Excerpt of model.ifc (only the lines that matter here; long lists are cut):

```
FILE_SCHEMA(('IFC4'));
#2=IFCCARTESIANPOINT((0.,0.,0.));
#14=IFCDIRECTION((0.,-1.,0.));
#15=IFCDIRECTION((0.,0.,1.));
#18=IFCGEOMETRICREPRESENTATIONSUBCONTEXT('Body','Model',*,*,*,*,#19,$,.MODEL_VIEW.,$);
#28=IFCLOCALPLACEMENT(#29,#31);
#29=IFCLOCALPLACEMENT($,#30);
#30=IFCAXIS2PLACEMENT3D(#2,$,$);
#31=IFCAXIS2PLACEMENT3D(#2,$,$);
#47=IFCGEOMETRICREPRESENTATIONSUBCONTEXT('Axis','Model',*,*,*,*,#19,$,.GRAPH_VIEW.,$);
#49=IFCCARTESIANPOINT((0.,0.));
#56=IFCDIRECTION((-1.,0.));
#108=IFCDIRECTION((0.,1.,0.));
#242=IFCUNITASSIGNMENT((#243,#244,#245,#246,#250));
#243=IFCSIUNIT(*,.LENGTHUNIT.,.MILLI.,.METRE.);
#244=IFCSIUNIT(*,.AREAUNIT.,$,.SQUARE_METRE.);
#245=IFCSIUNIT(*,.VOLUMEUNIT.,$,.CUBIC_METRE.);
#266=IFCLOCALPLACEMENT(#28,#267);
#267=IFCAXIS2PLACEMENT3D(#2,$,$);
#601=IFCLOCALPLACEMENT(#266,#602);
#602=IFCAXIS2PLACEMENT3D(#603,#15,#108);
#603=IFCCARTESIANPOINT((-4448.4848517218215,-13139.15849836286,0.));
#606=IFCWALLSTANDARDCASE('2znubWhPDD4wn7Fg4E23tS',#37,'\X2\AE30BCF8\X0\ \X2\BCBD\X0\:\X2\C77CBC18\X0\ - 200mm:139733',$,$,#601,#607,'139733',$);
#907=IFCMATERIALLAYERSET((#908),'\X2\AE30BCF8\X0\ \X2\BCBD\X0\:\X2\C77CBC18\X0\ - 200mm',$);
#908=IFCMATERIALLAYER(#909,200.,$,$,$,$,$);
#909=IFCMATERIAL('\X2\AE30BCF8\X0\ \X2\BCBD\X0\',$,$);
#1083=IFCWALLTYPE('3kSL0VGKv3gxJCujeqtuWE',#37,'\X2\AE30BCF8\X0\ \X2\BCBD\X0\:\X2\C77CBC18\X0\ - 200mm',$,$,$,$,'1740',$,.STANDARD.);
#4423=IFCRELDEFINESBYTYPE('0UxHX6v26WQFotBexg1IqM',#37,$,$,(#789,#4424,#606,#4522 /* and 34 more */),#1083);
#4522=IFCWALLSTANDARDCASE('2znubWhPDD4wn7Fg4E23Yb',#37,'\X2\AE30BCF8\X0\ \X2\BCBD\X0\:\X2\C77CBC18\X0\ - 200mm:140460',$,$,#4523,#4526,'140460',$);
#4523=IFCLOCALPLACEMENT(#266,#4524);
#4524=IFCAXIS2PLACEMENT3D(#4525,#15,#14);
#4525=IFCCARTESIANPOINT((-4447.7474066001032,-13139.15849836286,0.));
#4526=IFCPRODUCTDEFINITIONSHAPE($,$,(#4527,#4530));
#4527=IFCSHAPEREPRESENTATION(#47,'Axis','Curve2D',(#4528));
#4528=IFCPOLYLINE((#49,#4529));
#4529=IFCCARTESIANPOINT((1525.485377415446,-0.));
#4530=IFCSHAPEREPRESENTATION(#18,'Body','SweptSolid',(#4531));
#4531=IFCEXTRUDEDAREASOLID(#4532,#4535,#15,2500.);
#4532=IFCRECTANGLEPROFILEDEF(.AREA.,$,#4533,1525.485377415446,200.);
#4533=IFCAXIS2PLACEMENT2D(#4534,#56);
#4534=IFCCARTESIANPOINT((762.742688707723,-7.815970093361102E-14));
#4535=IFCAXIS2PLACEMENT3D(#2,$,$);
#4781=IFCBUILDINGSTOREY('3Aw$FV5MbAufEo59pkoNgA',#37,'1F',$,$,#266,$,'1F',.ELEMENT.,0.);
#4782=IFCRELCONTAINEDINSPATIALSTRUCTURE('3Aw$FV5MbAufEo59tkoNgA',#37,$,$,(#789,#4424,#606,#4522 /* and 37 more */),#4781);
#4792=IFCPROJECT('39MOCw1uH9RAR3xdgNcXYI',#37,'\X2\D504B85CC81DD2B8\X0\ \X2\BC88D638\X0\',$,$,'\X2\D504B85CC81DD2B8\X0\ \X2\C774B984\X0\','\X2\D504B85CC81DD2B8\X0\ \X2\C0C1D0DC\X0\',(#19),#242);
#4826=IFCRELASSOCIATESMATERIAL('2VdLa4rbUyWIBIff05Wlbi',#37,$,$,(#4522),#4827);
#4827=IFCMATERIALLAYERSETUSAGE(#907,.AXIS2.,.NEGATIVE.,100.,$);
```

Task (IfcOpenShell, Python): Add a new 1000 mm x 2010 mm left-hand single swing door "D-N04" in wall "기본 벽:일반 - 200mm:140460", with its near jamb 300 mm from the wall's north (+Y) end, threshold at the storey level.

```python
import numpy as np
import ifcopenshell
import ifcopenshell.api.feature
import ifcopenshell.api.geometry
import ifcopenshell.api.root
import ifcopenshell.api.spatial
import ifcopenshell.geom
import ifcopenshell.util.element
import ifcopenshell.util.placement
import ifcopenshell.util.representation
import ifcopenshell.util.shape
import ifcopenshell.util.unit

model = ifcopenshell.open("model.ifc")
unit_scale = ifcopenshell.util.unit.calculate_unit_scale(model)
settings = ifcopenshell.geom.settings()


def volume(element):
    """Net volume in cubic metres, openings subtracted."""
    shape = ifcopenshell.geom.create_shape(settings, element)
    return ifcopenshell.util.shape.get_volume(shape.geometry)


wall = model.by_id(4522)
storey = ifcopenshell.util.element.get_container(wall, ifc_class="IfcBuildingStorey")
context = ifcopenshell.util.representation.get_context(model, "Model", "Body", "MODEL_VIEW")
before = volume(wall)

width, height, from_end, sill = 1, 2.01, 0.3, 0.0  # metres

# The wall runs along its own X axis, and the end named is its -X end.
wall_shape = ifcopenshell.geom.create_shape(settings, wall)
x, y, z = ifcopenshell.util.shape.get_vertices(wall_shape.geometry).T
start = x.min() + from_end
face, thickness = float(y.min()), float(y.max() - y.min())
wall_matrix = ifcopenshell.util.placement.get_local_placement(wall.ObjectPlacement)
level = ifcopenshell.util.placement.get_local_placement(storey.ObjectPlacement)[2, 3]


def in_wall(x, y):
    """Placement at x, y metres in the wall's axes, at sill height."""
    matrix = wall_matrix.copy()
    matrix[:, 3] = wall_matrix @ np.array([x / unit_scale, y / unit_scale, 0.0, 1.0])
    matrix[2, 3] = level + sill / unit_scale
    return matrix


# Opening: a box that overshoots both wall faces by 50 mm.
opening = ifcopenshell.api.root.create_entity(model, ifc_class="IfcOpeningElement", predefined_type="OPENING")
box = ifcopenshell.api.geometry.add_wall_representation(
    model, context=context, length=width, height=height, thickness=thickness + 0.1
)
ifcopenshell.api.geometry.assign_representation(model, product=opening, representation=box)
ifcopenshell.api.geometry.edit_object_placement(model, product=opening, matrix=in_wall(start, face - 0.05), is_si=False)
ifcopenshell.api.feature.add_feature(model, feature=opening, element=wall)

door = ifcopenshell.api.root.create_entity(model, ifc_class="IfcDoor", name="D-N04", predefined_type="DOOR")
door.OverallWidth, door.OverallHeight = width / unit_scale, height / unit_scale
door.OperationType = "SINGLE_SWING_LEFT"
body = ifcopenshell.api.geometry.add_door_representation(
    model,
    context=context,
    overall_width=door.OverallWidth,
    overall_height=door.OverallHeight,
    operation_type="SINGLE_SWING_LEFT",
    lining_properties={"LiningDepth": thickness / unit_scale, "ThresholdDepth": thickness / unit_scale},
)
ifcopenshell.api.geometry.assign_representation(model, product=door, representation=body)
ifcopenshell.api.spatial.assign_container(model, products=[door], relating_structure=storey)
ifcopenshell.api.feature.add_filling(model, opening=opening, element=door)

# The lining spans the wall, so the door starts at the wall face.
ifcopenshell.api.geometry.edit_object_placement(model, product=door, matrix=in_wall(start, face), is_si=False)

after = volume(wall)

print(f"wall volume {before:.3f} -> {after:.3f} m3")

model.write("model_updated.ifc")
```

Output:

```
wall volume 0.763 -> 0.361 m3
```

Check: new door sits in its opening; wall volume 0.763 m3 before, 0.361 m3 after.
